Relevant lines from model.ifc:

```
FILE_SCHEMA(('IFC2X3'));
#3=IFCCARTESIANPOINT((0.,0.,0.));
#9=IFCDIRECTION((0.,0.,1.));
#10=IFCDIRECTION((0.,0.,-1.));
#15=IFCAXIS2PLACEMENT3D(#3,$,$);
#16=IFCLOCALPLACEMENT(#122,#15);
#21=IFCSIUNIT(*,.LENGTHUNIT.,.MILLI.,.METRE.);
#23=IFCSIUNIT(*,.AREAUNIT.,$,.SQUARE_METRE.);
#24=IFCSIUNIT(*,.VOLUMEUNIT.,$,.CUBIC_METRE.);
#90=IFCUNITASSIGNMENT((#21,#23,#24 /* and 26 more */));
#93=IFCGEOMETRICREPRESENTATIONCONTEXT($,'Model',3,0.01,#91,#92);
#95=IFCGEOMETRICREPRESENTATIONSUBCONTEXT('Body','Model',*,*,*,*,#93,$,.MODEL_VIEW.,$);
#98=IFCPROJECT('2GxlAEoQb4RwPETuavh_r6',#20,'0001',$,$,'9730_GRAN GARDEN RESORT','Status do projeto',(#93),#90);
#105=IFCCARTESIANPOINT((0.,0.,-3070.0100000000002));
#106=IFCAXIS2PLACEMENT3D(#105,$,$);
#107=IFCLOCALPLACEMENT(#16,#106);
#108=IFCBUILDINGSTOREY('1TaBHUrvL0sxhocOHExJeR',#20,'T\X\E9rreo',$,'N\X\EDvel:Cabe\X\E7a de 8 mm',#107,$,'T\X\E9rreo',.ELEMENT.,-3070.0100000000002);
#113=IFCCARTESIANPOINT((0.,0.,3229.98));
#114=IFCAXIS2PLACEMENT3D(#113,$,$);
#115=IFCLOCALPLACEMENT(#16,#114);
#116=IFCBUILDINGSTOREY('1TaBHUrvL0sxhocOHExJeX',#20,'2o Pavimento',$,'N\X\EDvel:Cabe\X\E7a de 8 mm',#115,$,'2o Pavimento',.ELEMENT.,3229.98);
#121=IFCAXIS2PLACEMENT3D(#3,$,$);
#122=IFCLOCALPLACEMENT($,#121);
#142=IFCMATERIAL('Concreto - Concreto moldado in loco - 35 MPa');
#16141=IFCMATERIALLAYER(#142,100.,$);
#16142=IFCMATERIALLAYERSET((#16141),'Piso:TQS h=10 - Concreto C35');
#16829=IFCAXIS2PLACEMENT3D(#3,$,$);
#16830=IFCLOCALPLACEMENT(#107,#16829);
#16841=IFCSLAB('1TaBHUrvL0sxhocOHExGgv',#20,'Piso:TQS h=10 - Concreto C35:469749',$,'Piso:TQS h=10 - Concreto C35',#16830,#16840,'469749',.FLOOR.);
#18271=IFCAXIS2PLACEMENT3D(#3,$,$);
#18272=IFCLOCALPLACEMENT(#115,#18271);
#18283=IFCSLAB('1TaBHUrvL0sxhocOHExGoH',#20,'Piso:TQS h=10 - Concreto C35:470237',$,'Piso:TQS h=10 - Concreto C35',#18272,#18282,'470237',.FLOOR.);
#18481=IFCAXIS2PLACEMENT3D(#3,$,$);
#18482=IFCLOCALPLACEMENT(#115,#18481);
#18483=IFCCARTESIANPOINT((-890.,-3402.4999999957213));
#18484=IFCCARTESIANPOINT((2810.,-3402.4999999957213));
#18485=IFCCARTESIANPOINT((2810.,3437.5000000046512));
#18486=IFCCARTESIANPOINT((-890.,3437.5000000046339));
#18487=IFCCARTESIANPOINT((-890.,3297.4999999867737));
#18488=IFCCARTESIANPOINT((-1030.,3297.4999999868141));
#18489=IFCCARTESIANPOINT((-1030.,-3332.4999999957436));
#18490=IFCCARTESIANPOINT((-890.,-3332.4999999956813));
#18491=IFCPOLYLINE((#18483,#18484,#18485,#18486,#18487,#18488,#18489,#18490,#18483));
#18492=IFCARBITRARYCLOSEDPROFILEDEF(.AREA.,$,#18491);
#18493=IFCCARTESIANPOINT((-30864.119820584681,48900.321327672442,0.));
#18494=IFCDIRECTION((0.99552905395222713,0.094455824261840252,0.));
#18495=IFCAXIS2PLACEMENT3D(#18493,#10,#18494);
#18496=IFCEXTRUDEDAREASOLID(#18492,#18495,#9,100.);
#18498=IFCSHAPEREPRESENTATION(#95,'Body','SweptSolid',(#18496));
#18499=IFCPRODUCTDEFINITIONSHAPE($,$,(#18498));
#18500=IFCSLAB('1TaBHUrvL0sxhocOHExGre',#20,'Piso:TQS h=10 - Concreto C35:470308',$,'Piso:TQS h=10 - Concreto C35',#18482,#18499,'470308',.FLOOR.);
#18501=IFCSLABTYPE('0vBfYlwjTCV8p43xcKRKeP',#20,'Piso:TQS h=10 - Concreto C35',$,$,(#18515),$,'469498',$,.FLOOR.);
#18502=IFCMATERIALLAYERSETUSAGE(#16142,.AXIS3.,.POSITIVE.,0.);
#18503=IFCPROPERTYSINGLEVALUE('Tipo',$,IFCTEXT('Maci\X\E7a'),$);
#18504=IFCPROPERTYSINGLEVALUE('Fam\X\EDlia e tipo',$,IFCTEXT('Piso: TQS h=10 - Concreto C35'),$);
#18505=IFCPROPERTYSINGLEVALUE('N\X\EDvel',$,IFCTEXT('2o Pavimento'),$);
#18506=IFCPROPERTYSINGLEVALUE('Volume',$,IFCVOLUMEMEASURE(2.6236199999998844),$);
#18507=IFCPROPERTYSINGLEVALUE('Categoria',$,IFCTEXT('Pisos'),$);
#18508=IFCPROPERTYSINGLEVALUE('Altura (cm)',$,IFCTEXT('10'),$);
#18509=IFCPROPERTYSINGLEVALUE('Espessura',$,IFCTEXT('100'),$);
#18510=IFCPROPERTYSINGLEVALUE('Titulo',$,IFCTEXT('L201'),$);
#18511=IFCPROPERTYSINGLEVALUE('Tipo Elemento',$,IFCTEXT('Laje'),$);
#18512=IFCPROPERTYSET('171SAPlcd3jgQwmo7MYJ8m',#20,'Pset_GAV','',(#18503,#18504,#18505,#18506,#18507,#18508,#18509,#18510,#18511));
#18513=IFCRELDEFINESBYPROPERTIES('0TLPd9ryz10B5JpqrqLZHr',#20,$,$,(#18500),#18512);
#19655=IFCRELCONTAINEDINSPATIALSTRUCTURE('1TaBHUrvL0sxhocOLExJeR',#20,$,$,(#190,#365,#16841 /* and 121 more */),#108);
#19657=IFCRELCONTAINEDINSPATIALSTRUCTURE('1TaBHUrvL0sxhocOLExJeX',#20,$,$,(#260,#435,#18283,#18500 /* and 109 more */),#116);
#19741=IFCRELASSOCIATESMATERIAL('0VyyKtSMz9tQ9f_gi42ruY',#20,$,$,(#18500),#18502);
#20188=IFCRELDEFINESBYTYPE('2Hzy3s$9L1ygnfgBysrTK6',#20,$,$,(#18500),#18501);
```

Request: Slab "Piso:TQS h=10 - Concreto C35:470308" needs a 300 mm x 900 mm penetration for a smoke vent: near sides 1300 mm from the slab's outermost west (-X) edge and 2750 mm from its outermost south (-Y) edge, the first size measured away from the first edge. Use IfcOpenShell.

```python
import numpy as np
import ifcopenshell
import ifcopenshell.api.feature
import ifcopenshell.api.geometry
import ifcopenshell.api.pset
import ifcopenshell.api.root
import ifcopenshell.geom
import ifcopenshell.util.element
import ifcopenshell.util.placement
import ifcopenshell.util.representation
import ifcopenshell.util.shape
import ifcopenshell.util.unit

model = ifcopenshell.open("model.ifc")
unit_scale = ifcopenshell.util.unit.calculate_unit_scale(model)
volume_scale = ifcopenshell.util.unit.calculate_unit_scale(model, "VOLUMEUNIT")
settings = ifcopenshell.geom.settings()


def volume(element):
    """Net volume in cubic metres, openings subtracted."""
    shape = ifcopenshell.geom.create_shape(settings, element)
    return ifcopenshell.util.shape.get_volume(shape.geometry)


slab = model.by_guid("1TaBHUrvL0sxhocOHExGre")
before = volume(slab)

# Extent in the slab's own axes, in metres. The edges named are its -X and -Y sides.
slab_shape = ifcopenshell.geom.create_shape(settings, slab)
vertices = ifcopenshell.util.shape.get_vertices(slab_shape.geometry)
x_min, y_min, bottom = vertices.min(axis=0)
top = vertices[:, 2].max()

opening = ifcopenshell.api.root.create_entity(model, ifc_class="IfcOpeningElement", name="Smoke vent opening")
context = ifcopenshell.util.representation.get_context(model, "Model", "Body", "MODEL_VIEW")
width, depth = 0.3, 0.9
outline = [(0.0, 0.0), (width, 0.0), (width, depth), (0.0, depth), (0.0, 0.0)]
# Overshoot both faces by 50 mm so the cut is clean.
shape = ifcopenshell.api.geometry.add_slab_representation(
    model, context=context, depth=top - bottom + 0.1, polyline=outline
)
ifcopenshell.api.geometry.assign_representation(model, product=opening, representation=shape)

matrix = ifcopenshell.util.placement.get_local_placement(slab.ObjectPlacement)
matrix[:, 3] = matrix @ np.append(np.array([x_min + 1.3, y_min + 2.75, bottom - 0.05]) / unit_scale, 1.0)
ifcopenshell.api.geometry.edit_object_placement(model, product=opening, matrix=matrix, is_si=False)
ifcopenshell.api.feature.add_feature(model, feature=opening, element=slab)

after = volume(slab)

# Update the slab's stored quantities.
pset = model.by_id(ifcopenshell.util.element.get_pset(slab, "Pset_GAV", should_inherit=False)["id"])
ifcopenshell.api.pset.edit_pset(model, pset=pset, properties={
    "Volume": model.create_entity("IfcVolumeMeasure", after / volume_scale),
})

print(f"slab volume {before:.3f} -> {after:.3f} m3")

model.write("model_updated.ifc")
```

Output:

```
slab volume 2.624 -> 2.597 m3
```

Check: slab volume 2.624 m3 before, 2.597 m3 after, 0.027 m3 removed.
